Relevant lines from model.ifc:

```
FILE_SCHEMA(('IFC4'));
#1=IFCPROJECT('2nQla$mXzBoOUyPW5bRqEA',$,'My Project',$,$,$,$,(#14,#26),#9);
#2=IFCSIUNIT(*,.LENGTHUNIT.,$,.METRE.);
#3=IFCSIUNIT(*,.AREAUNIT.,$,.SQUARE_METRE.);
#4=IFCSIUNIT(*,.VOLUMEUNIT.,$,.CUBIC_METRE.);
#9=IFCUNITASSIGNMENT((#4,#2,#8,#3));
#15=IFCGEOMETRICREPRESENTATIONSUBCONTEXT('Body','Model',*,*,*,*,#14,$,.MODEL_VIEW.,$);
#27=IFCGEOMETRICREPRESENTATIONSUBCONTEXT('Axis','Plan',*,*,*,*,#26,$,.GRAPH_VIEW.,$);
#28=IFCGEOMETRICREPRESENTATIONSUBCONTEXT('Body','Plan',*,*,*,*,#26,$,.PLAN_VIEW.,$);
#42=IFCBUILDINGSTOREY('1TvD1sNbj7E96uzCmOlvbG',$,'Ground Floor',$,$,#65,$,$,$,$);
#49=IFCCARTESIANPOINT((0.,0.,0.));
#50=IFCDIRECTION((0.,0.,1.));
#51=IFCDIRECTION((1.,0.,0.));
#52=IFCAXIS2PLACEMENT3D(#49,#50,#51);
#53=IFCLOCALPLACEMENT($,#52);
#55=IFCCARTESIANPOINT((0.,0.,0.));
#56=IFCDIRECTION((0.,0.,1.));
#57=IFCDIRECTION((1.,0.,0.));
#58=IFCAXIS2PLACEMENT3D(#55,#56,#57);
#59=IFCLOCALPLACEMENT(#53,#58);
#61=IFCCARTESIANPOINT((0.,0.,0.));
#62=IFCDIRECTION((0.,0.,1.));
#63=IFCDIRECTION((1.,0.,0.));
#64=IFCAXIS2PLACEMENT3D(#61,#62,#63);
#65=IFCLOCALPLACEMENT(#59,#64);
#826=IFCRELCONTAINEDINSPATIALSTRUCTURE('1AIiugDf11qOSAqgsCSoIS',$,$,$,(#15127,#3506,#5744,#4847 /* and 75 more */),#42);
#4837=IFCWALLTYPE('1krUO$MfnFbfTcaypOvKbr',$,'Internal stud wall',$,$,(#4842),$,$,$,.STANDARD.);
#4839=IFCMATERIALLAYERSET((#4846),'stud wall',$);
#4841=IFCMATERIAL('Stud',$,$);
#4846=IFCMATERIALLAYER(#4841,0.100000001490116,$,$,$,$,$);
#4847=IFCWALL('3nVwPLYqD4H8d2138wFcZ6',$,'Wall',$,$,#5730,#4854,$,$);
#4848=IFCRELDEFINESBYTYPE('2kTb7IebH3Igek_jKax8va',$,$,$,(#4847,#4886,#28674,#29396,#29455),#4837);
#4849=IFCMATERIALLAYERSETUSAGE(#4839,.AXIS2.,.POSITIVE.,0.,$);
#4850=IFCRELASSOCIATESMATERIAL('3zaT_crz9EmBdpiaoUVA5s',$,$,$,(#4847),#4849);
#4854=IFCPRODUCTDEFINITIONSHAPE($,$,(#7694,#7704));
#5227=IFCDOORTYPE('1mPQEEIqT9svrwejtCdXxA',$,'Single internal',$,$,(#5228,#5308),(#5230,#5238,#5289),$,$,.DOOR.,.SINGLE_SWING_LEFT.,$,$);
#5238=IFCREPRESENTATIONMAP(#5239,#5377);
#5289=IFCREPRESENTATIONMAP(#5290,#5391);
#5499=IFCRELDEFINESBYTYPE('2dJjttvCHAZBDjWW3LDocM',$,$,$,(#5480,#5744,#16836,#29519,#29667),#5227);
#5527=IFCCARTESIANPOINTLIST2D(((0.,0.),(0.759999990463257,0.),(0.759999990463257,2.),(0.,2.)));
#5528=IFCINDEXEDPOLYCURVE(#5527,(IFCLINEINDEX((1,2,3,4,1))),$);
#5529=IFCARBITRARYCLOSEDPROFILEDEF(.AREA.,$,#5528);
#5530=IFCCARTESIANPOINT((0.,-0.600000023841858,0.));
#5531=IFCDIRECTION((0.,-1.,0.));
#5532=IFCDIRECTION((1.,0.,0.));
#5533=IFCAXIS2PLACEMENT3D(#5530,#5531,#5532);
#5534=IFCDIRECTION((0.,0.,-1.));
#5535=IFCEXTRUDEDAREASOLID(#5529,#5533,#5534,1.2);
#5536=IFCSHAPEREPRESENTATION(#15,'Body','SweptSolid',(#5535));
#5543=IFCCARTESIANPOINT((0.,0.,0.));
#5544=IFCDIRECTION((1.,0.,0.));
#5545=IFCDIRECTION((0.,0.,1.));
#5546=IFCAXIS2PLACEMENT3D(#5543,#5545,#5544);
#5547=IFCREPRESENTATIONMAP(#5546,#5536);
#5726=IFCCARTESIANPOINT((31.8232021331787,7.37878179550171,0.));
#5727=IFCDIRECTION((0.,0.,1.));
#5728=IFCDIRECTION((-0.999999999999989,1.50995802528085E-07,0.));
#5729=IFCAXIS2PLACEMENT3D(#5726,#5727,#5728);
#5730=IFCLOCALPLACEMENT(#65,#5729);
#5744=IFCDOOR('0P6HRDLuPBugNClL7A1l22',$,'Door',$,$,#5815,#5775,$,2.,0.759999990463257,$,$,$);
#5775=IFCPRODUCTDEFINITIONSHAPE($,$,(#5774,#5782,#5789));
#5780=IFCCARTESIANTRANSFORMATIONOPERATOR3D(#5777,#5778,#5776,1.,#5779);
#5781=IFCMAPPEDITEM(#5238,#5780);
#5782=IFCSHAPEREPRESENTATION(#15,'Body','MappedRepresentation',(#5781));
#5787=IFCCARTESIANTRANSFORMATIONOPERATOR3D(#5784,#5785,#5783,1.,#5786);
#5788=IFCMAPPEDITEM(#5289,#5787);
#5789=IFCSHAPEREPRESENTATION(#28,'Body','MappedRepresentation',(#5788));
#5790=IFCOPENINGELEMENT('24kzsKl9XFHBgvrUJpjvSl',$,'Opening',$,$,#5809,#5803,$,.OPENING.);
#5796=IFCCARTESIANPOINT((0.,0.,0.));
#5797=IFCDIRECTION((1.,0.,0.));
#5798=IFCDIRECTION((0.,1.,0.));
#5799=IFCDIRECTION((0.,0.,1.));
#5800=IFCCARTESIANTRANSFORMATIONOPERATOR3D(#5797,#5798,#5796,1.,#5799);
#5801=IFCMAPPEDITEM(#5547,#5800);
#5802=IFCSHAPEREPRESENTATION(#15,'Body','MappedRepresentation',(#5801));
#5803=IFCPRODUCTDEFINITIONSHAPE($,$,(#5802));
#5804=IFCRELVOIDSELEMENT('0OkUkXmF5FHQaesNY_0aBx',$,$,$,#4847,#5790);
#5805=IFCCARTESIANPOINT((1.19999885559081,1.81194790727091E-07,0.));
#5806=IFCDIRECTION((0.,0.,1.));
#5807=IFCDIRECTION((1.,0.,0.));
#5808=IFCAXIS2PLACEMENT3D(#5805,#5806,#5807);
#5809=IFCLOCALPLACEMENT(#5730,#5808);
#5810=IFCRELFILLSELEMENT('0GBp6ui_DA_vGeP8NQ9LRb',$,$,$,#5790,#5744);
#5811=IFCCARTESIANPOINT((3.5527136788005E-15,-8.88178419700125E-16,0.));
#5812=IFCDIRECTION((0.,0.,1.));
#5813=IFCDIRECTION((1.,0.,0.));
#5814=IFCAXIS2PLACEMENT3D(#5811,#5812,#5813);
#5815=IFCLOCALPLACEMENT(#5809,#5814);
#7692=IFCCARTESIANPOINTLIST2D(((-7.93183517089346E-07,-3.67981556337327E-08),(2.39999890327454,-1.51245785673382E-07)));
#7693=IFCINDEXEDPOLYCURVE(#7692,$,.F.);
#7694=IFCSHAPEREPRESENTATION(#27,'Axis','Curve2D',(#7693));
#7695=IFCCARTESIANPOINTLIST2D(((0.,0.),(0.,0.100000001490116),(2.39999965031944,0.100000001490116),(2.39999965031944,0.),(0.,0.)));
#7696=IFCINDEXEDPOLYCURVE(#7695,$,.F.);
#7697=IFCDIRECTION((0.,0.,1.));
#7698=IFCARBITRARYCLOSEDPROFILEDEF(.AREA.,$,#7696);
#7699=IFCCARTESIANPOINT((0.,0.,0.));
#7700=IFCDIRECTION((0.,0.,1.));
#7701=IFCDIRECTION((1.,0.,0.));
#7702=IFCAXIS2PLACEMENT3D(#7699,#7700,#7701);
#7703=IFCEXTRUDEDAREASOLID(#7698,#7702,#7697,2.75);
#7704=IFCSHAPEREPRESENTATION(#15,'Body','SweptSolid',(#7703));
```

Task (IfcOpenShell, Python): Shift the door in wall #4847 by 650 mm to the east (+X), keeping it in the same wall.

```python
import ifcopenshell
import ifcopenshell.api.geometry
import ifcopenshell.util.placement
import ifcopenshell.util.unit

model = ifcopenshell.open("model.ifc")
unit_scale = ifcopenshell.util.unit.calculate_unit_scale(model)

door = model.by_guid("0P6HRDLuPBugNClL7A1l22")
opening = door.FillsVoids[0].RelatingOpeningElement
wall = opening.VoidsElements[0].RelatingBuildingElement

wall_matrix = ifcopenshell.util.placement.get_local_placement(wall.ObjectPlacement)
shift = wall_matrix[:3, 0] * -0.65 / unit_scale
before = ifcopenshell.util.placement.get_local_placement(door.ObjectPlacement)[:3, 3].copy()

# The door is placed relative to its opening, so it follows when the opening moves.
matrix = ifcopenshell.util.placement.get_local_placement(opening.ObjectPlacement)
matrix[:3, 3] += shift
ifcopenshell.api.geometry.edit_object_placement(
    model, product=opening, matrix=matrix, is_si=False, should_transform_children=True
)

after = ifcopenshell.util.placement.get_local_placement(door.ObjectPlacement)[:3, 3]
print("door moved by", (after - before).round(3) + 0.0)

model.write("model_updated.ifc")
```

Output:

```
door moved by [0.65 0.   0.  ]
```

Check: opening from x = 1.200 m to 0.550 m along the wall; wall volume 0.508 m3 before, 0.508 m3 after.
